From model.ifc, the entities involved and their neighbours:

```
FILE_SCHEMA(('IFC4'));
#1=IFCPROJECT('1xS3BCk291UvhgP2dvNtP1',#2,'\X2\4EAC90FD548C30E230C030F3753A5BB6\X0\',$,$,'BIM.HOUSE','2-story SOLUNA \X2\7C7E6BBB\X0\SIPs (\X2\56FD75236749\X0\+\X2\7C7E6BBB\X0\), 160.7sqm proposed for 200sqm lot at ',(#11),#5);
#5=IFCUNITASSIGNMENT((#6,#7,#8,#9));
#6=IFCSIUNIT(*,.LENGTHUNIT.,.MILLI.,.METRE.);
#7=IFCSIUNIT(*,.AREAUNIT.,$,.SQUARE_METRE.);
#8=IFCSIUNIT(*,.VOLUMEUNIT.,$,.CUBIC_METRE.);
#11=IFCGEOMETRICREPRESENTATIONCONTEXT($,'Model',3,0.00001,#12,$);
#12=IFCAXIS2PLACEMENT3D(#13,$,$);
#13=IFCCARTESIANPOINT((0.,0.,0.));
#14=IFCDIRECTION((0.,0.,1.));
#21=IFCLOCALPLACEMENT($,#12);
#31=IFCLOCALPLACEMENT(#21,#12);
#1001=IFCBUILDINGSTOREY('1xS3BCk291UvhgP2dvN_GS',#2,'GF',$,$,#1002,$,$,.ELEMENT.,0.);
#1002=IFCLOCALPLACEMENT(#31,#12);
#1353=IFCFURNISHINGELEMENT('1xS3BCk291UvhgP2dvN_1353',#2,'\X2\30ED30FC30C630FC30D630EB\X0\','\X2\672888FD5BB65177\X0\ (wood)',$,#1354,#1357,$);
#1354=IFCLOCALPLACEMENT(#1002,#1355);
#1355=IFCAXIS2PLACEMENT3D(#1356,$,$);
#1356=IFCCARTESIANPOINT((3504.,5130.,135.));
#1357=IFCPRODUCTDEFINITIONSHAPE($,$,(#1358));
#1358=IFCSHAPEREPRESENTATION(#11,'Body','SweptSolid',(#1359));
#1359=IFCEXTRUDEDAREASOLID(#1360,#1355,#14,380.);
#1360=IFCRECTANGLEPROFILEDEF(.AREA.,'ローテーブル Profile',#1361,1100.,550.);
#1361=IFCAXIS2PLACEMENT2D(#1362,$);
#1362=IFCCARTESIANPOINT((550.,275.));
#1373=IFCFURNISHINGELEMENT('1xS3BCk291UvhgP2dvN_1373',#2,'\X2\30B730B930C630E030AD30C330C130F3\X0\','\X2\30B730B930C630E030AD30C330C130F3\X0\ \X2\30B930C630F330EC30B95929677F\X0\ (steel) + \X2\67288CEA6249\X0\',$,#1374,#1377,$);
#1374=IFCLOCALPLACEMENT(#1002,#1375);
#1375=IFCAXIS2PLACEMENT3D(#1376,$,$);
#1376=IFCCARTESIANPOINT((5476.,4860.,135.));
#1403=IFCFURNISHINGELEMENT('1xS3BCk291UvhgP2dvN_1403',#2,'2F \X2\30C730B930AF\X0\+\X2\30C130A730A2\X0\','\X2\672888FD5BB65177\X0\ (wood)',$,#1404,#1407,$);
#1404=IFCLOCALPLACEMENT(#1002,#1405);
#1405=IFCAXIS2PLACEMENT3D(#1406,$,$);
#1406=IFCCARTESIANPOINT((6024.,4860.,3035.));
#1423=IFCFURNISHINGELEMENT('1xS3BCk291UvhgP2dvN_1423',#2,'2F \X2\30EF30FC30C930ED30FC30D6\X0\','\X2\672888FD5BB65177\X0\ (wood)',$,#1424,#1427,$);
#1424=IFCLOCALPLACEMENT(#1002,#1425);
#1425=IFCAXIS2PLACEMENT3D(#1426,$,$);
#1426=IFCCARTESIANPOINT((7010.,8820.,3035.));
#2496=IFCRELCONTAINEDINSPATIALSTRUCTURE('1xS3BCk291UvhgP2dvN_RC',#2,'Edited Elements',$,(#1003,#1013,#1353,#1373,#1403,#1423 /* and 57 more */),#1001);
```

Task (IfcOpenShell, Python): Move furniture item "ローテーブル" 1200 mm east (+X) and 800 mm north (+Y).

```python
import ifcopenshell
import ifcopenshell.api.geometry
import ifcopenshell.util.placement

model = ifcopenshell.open("model.ifc")

item = model.by_guid("1xS3BCk291UvhgP2dvN_1353")
matrix = ifcopenshell.util.placement.get_local_placement(item.ObjectPlacement)
matrix[0, 3] += 1200.0
matrix[1, 3] += 800.0
ifcopenshell.api.geometry.edit_object_placement(model, product=item, matrix=matrix, is_si=False)

print(ifcopenshell.util.placement.get_local_placement(item.ObjectPlacement).round(3) + 0.0)

model.write("model_rev.ifc")
```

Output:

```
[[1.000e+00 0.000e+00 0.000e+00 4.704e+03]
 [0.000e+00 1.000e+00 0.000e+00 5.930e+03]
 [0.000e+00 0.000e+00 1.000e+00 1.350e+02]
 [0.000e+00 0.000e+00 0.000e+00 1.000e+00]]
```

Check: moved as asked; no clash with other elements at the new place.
